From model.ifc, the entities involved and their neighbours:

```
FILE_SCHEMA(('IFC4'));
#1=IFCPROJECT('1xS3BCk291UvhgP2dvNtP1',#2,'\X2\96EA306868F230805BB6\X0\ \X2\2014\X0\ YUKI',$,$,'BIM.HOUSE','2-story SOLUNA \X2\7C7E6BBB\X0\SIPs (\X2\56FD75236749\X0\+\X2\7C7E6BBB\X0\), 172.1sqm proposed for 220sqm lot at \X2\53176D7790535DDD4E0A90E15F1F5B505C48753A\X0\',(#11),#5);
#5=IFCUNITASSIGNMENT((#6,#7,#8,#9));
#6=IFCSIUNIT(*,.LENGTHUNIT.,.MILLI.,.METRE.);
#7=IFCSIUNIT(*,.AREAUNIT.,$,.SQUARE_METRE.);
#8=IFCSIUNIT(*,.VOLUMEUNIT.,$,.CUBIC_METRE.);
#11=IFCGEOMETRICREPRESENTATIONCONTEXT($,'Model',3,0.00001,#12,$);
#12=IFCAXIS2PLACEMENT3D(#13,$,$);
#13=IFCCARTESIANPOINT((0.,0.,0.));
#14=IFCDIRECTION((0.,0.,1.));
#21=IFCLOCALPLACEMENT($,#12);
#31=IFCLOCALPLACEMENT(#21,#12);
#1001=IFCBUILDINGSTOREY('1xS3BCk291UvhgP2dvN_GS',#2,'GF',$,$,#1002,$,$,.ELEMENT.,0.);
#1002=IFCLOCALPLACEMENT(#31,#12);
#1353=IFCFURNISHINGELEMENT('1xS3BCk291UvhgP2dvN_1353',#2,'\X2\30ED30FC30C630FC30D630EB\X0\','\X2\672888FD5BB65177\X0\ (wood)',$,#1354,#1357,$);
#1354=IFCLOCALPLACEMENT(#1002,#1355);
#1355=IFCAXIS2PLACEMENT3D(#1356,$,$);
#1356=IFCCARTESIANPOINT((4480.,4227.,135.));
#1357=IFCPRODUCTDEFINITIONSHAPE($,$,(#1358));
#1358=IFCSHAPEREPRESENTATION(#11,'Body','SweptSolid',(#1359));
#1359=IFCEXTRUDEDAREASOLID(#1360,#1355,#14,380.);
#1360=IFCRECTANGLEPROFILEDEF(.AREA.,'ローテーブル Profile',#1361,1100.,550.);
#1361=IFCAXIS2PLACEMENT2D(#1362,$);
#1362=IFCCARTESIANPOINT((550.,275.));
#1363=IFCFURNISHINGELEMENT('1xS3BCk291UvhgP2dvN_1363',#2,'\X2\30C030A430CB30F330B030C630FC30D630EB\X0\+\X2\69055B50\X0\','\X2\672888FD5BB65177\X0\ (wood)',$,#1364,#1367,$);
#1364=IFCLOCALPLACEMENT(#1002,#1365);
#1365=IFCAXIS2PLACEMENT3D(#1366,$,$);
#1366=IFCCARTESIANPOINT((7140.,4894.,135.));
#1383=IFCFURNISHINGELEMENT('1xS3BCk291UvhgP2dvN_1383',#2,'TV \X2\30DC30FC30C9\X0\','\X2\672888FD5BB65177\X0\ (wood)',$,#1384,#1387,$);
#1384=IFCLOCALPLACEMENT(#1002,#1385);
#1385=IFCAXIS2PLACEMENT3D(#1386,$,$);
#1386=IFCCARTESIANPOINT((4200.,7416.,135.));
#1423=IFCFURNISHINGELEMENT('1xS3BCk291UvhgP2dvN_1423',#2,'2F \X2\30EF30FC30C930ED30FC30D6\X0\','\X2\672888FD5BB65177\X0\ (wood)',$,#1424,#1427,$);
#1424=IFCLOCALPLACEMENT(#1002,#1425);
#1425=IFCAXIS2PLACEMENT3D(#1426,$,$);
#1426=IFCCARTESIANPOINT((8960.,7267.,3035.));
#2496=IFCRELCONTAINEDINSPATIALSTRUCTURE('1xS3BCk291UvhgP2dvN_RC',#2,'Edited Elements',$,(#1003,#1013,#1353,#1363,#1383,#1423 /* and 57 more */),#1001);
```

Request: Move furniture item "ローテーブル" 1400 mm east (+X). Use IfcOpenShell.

```python
import ifcopenshell
import ifcopenshell.api.geometry
import ifcopenshell.util.placement

model = ifcopenshell.open("model.ifc")

item = model.by_guid("1xS3BCk291UvhgP2dvN_1353")
matrix = ifcopenshell.util.placement.get_local_placement(item.ObjectPlacement)
matrix[0, 3] += 1400.0
ifcopenshell.api.geometry.edit_object_placement(model, product=item, matrix=matrix, is_si=False)

print(ifcopenshell.util.placement.get_local_placement(item.ObjectPlacement).round(3) + 0.0)

model.write("model_rev.ifc")
```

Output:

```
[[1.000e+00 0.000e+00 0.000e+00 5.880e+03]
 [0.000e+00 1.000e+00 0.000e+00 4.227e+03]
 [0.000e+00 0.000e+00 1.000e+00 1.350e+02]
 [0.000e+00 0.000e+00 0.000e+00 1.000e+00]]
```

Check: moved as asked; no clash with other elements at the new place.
